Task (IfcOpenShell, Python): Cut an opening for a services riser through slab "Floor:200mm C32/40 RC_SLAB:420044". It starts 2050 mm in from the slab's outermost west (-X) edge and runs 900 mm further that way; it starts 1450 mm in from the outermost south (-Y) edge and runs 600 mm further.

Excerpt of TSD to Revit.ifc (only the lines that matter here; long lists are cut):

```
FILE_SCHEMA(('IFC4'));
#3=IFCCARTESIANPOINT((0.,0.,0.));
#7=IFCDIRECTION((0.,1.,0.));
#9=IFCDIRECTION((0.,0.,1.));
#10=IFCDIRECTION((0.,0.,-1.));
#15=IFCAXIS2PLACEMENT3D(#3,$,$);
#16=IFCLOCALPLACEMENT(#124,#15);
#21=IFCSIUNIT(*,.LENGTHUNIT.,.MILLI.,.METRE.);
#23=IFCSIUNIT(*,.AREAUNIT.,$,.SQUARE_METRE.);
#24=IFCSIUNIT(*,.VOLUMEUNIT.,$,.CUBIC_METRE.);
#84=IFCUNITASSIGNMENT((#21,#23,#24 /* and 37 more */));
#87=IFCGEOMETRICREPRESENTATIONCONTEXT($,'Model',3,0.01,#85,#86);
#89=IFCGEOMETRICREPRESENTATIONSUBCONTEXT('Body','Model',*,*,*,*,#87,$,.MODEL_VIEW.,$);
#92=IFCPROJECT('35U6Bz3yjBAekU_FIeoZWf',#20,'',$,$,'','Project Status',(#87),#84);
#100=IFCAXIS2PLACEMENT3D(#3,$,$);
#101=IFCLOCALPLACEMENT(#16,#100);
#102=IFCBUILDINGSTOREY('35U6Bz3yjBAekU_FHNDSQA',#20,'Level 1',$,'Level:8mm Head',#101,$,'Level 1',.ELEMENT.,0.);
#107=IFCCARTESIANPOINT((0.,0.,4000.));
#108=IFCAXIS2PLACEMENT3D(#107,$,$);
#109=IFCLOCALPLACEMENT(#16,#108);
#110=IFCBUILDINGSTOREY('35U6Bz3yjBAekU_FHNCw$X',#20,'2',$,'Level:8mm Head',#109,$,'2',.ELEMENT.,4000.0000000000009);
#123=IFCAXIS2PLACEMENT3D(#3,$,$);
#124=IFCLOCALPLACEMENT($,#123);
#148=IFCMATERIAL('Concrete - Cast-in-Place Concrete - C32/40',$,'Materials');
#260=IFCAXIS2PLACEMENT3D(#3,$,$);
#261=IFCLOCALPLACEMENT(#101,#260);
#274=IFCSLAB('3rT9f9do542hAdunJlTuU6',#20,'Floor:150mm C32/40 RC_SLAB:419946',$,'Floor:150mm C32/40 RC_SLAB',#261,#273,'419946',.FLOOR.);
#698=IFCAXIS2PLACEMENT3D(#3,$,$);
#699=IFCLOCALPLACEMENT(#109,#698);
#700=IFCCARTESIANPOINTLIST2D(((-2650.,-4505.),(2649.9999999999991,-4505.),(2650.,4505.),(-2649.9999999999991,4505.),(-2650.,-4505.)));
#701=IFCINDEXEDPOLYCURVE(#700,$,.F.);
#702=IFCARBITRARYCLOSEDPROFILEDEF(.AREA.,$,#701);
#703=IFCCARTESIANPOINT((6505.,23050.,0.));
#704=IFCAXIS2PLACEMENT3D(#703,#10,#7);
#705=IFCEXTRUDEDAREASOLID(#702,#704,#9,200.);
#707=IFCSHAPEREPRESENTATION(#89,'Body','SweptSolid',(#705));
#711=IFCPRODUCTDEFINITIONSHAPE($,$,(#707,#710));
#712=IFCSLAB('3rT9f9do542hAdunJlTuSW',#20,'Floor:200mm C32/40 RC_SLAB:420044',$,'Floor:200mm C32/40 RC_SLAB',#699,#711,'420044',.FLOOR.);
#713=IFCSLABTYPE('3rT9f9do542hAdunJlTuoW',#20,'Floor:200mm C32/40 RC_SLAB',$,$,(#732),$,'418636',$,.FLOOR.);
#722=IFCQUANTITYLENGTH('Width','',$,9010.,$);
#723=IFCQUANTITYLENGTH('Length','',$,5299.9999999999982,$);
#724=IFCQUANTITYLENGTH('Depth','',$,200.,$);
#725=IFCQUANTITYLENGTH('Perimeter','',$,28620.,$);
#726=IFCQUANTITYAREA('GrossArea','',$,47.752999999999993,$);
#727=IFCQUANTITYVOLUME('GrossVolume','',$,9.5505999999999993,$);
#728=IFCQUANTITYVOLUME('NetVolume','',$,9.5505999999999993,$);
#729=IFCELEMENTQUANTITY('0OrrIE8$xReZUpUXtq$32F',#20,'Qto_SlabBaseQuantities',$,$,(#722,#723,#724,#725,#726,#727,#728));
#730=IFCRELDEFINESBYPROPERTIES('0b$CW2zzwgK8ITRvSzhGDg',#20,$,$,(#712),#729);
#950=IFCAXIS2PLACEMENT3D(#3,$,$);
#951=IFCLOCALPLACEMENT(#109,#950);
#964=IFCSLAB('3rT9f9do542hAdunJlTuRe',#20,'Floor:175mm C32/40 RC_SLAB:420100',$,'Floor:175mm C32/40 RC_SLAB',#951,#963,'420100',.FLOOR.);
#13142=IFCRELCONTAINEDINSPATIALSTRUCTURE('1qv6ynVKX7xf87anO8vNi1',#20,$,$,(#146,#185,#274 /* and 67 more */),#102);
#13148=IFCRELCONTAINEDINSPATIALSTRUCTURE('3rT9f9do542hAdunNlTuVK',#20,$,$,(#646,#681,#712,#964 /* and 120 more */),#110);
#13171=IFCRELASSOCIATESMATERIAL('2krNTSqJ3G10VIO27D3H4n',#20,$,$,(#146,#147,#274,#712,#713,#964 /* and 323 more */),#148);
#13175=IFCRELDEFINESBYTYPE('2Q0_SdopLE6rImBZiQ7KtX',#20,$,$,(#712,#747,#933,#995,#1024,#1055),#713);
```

```python
import numpy as np
import ifcopenshell
import ifcopenshell.api.feature
import ifcopenshell.api.geometry
import ifcopenshell.api.pset
import ifcopenshell.api.root
import ifcopenshell.geom
import ifcopenshell.util.element
import ifcopenshell.util.placement
import ifcopenshell.util.representation
import ifcopenshell.util.shape
import ifcopenshell.util.unit

model = ifcopenshell.open("TSD to Revit.ifc")
unit_scale = ifcopenshell.util.unit.calculate_unit_scale(model)
volume_scale = ifcopenshell.util.unit.calculate_unit_scale(model, "VOLUMEUNIT")
settings = ifcopenshell.geom.settings()


def volume(element):
    """Net volume in cubic metres, openings subtracted."""
    shape = ifcopenshell.geom.create_shape(settings, element)
    return ifcopenshell.util.shape.get_volume(shape.geometry)


slab = model.by_guid("3rT9f9do542hAdunJlTuSW")
before = volume(slab)

# Extent in the slab's own axes, in metres. The edges named are its -X and -Y sides.
slab_shape = ifcopenshell.geom.create_shape(settings, slab)
vertices = ifcopenshell.util.shape.get_vertices(slab_shape.geometry)
x_min, y_min, bottom = vertices.min(axis=0)
top = vertices[:, 2].max()

opening = ifcopenshell.api.root.create_entity(model, ifc_class="IfcOpeningElement", name="Services riser opening", predefined_type="OPENING")
context = ifcopenshell.util.representation.get_context(model, "Model", "Body", "MODEL_VIEW")
width, depth = 0.9, 0.6
outline = [(0.0, 0.0), (width, 0.0), (width, depth), (0.0, depth), (0.0, 0.0)]
# Overshoot both faces by 50 mm so the cut is clean.
shape = ifcopenshell.api.geometry.add_slab_representation(
    model, context=context, depth=top - bottom + 0.1, polyline=outline
)
ifcopenshell.api.geometry.assign_representation(model, product=opening, representation=shape)

matrix = ifcopenshell.util.placement.get_local_placement(slab.ObjectPlacement)
matrix[:, 3] = matrix @ np.append(np.array([x_min + 2.05, y_min + 1.45, bottom - 0.05]) / unit_scale, 1.0)
ifcopenshell.api.geometry.edit_object_placement(model, product=opening, matrix=matrix, is_si=False)
ifcopenshell.api.feature.add_feature(model, feature=opening, element=slab)

after = volume(slab)

# Update the slab's stored quantities.
qto = model.by_id(ifcopenshell.util.element.get_pset(slab, "Qto_SlabBaseQuantities", should_inherit=False)["id"])
ifcopenshell.api.pset.edit_qto(model, qto=qto, properties={"NetVolume": after / volume_scale})

print(f"slab volume {before:.3f} -> {after:.3f} m3")

model.write("TSD to Revit_rev.ifc")
```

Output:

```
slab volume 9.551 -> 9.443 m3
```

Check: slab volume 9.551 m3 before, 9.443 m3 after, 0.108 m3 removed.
